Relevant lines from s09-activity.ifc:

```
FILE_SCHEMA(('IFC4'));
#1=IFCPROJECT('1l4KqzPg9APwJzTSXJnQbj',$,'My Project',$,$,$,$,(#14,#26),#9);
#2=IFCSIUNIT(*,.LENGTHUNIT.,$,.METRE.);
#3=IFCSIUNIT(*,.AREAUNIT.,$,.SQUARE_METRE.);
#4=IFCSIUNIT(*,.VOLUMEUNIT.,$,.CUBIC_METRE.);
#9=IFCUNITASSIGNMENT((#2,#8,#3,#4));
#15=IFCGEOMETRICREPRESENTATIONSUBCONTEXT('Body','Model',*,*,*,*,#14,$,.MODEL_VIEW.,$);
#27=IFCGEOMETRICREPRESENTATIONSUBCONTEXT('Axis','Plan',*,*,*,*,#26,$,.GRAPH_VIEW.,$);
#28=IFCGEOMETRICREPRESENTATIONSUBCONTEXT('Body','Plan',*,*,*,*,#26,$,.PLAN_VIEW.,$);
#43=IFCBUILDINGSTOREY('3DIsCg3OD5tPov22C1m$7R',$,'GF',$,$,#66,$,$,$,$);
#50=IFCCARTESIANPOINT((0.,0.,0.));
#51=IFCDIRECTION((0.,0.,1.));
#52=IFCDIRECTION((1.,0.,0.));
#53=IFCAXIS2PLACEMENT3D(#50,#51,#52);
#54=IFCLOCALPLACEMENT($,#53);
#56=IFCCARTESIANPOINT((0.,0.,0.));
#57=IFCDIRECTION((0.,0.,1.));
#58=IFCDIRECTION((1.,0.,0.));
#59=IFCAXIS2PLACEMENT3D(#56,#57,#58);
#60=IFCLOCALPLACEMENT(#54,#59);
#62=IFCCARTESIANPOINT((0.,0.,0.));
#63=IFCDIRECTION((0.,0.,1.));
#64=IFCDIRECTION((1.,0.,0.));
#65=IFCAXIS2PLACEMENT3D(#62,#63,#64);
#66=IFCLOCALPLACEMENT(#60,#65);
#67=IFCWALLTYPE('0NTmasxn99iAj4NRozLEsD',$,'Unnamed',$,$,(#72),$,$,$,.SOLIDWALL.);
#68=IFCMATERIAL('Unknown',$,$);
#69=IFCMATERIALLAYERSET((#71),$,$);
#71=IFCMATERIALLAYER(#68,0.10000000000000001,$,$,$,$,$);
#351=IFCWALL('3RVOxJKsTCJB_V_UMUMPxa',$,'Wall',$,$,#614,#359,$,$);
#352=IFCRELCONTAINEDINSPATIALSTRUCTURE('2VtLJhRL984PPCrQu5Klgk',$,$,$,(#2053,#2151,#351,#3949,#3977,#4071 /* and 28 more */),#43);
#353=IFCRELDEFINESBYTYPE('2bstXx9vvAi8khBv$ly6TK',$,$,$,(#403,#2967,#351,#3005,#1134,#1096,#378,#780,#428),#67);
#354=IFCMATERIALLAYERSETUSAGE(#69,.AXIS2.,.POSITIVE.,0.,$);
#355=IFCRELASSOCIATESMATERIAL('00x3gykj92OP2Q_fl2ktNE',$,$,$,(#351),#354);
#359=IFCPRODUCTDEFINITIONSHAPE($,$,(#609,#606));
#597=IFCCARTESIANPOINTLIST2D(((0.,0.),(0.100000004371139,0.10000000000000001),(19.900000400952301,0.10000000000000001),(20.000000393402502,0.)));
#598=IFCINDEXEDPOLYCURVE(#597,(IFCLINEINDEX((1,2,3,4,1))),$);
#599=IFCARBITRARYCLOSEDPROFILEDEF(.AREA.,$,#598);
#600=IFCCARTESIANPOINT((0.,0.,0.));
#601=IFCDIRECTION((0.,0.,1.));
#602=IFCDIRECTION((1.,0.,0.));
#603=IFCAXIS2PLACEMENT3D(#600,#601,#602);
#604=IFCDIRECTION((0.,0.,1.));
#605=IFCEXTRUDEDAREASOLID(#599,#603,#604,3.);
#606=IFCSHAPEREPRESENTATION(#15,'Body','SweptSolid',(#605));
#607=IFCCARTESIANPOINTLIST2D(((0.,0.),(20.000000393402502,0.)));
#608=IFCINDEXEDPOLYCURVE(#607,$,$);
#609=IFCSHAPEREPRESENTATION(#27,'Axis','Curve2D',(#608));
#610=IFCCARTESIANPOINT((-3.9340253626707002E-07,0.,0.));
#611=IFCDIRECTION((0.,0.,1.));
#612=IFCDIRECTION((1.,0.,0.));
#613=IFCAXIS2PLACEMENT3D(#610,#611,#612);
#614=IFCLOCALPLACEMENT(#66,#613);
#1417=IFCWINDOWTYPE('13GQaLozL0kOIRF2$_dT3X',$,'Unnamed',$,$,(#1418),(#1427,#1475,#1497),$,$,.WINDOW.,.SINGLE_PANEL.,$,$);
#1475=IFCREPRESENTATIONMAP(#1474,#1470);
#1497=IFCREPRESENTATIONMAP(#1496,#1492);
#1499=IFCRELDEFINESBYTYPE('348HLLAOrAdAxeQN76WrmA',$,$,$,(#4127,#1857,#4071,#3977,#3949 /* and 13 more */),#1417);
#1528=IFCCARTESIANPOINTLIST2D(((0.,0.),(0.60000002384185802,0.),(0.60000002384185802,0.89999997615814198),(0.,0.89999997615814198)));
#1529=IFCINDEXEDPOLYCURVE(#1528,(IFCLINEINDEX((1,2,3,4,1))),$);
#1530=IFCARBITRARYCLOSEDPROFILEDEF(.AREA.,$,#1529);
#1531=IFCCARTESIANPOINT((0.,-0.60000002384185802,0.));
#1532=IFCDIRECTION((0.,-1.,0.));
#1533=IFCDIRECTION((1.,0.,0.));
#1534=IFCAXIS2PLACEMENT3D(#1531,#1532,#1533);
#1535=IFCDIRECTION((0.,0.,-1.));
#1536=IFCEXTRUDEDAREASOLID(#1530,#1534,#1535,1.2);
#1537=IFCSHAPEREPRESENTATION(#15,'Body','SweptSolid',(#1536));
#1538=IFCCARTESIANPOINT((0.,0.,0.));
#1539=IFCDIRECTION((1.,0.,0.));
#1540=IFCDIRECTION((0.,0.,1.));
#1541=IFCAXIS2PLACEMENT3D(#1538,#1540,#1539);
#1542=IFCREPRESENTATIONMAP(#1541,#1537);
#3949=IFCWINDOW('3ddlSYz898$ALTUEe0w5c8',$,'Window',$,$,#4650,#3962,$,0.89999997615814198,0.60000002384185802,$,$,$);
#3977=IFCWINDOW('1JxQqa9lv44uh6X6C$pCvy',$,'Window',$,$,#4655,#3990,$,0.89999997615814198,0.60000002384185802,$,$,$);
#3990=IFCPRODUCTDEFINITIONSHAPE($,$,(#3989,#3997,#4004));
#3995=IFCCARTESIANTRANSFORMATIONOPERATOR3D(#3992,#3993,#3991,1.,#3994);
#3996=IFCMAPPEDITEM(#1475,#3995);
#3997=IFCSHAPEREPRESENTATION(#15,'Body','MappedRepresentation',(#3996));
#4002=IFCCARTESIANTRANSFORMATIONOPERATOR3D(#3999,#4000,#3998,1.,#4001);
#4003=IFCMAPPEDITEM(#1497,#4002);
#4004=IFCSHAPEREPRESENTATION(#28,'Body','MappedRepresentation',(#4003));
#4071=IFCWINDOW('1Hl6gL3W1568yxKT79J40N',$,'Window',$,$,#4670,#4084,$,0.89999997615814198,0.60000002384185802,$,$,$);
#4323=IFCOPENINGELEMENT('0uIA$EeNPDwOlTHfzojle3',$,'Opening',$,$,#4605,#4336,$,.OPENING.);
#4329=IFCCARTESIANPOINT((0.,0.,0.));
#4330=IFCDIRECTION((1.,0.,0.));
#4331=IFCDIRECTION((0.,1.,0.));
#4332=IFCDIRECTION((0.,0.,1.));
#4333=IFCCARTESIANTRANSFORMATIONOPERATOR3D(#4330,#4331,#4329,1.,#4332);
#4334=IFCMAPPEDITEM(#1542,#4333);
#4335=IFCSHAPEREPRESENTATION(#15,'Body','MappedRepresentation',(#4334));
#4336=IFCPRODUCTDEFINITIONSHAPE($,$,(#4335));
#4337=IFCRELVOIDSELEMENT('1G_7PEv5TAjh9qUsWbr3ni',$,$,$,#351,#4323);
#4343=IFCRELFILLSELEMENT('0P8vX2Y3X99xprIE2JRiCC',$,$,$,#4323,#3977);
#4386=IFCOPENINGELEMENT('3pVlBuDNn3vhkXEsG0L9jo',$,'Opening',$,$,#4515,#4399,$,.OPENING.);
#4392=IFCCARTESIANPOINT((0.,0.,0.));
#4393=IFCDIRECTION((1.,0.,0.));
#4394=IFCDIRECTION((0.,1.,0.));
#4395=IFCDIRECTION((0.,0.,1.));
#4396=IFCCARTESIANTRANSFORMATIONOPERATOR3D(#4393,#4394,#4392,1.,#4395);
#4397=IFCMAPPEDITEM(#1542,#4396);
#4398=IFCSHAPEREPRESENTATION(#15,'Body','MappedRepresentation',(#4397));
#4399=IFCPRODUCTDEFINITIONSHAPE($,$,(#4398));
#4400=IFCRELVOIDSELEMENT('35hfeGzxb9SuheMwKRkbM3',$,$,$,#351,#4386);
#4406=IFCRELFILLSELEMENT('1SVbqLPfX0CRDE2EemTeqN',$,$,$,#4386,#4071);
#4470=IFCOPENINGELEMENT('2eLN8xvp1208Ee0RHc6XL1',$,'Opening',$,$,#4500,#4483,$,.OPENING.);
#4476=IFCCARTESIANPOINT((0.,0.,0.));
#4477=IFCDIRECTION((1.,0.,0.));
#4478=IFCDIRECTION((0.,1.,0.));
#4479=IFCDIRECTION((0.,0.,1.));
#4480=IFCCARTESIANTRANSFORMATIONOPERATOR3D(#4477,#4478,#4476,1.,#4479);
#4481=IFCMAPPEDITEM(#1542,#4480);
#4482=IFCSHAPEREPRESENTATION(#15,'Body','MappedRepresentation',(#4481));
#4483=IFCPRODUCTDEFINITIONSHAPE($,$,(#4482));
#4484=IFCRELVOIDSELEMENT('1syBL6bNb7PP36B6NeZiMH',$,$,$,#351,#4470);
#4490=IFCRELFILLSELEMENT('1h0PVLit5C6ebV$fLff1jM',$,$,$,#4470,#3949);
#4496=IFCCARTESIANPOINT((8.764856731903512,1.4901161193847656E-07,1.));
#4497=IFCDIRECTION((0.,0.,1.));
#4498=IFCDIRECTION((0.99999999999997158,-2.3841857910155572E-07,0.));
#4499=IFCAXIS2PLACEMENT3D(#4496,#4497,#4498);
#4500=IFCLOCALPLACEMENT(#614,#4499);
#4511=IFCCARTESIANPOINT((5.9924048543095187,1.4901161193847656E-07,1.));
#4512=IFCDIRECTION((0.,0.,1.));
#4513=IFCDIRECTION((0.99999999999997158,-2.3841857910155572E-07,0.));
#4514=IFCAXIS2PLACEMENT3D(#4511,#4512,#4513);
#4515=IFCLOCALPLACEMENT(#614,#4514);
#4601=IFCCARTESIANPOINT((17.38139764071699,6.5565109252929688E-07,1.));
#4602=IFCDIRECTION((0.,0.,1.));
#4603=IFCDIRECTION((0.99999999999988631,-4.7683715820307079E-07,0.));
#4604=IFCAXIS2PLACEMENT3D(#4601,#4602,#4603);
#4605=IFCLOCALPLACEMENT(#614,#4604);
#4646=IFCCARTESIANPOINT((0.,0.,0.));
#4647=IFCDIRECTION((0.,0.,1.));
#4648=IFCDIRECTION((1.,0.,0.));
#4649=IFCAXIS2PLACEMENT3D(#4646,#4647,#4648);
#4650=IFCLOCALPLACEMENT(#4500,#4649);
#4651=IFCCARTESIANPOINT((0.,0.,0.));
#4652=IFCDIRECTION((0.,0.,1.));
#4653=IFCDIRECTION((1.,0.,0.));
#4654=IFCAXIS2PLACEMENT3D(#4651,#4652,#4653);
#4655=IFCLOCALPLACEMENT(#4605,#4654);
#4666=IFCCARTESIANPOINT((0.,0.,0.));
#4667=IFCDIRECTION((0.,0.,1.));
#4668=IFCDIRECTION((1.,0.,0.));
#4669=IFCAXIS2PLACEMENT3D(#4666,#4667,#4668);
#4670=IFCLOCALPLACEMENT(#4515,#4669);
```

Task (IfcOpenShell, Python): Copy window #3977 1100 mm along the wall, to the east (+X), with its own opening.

```python
import ifcopenshell
import ifcopenshell.api.feature
import ifcopenshell.api.geometry
import ifcopenshell.api.root
import ifcopenshell.geom
import ifcopenshell.util.element
import ifcopenshell.util.placement
import ifcopenshell.util.shape
import ifcopenshell.util.unit

model = ifcopenshell.open("s09-activity.ifc")
unit_scale = ifcopenshell.util.unit.calculate_unit_scale(model)
settings = ifcopenshell.geom.settings()


def volume(element):
    """Net volume in cubic metres, openings subtracted."""
    shape = ifcopenshell.geom.create_shape(settings, element)
    return ifcopenshell.util.shape.get_volume(shape.geometry)


window = model.by_guid("1JxQqa9lv44uh6X6C$pCvy")
opening = window.FillsVoids[0].RelatingOpeningElement
wall = opening.VoidsElements[0].RelatingBuildingElement
before = volume(wall)
shift = ifcopenshell.util.placement.get_local_placement(wall.ObjectPlacement)[:3, 0] * 1.1 / unit_scale

# copy_class copies the void relationship, type, container and properties, but no geometry.
new_opening = ifcopenshell.api.root.copy_class(model, product=opening)
new_opening.Representation = ifcopenshell.util.element.copy_deep(
    model, opening.Representation, exclude=["IfcGeometricRepresentationContext", "IfcRepresentationMap"]
)
new_window = ifcopenshell.api.root.copy_class(model, product=window)
new_window.Representation = ifcopenshell.util.element.copy_deep(
    model, window.Representation, exclude=["IfcGeometricRepresentationContext", "IfcRepresentationMap"]
)
ifcopenshell.api.feature.add_filling(model, opening=new_opening, element=new_window)

for old, new in ((opening, new_opening), (window, new_window)):
    matrix = ifcopenshell.util.placement.get_local_placement(old.ObjectPlacement)
    matrix[:3, 3] += shift
    ifcopenshell.api.geometry.edit_object_placement(model, product=new, matrix=matrix, is_si=False)

after = volume(wall)

print(f"wall volume {before:.3f} -> {after:.3f} m3")

model.write("s09-activity_edited.ifc")
```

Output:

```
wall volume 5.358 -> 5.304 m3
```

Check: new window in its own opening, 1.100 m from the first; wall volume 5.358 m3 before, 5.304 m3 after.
